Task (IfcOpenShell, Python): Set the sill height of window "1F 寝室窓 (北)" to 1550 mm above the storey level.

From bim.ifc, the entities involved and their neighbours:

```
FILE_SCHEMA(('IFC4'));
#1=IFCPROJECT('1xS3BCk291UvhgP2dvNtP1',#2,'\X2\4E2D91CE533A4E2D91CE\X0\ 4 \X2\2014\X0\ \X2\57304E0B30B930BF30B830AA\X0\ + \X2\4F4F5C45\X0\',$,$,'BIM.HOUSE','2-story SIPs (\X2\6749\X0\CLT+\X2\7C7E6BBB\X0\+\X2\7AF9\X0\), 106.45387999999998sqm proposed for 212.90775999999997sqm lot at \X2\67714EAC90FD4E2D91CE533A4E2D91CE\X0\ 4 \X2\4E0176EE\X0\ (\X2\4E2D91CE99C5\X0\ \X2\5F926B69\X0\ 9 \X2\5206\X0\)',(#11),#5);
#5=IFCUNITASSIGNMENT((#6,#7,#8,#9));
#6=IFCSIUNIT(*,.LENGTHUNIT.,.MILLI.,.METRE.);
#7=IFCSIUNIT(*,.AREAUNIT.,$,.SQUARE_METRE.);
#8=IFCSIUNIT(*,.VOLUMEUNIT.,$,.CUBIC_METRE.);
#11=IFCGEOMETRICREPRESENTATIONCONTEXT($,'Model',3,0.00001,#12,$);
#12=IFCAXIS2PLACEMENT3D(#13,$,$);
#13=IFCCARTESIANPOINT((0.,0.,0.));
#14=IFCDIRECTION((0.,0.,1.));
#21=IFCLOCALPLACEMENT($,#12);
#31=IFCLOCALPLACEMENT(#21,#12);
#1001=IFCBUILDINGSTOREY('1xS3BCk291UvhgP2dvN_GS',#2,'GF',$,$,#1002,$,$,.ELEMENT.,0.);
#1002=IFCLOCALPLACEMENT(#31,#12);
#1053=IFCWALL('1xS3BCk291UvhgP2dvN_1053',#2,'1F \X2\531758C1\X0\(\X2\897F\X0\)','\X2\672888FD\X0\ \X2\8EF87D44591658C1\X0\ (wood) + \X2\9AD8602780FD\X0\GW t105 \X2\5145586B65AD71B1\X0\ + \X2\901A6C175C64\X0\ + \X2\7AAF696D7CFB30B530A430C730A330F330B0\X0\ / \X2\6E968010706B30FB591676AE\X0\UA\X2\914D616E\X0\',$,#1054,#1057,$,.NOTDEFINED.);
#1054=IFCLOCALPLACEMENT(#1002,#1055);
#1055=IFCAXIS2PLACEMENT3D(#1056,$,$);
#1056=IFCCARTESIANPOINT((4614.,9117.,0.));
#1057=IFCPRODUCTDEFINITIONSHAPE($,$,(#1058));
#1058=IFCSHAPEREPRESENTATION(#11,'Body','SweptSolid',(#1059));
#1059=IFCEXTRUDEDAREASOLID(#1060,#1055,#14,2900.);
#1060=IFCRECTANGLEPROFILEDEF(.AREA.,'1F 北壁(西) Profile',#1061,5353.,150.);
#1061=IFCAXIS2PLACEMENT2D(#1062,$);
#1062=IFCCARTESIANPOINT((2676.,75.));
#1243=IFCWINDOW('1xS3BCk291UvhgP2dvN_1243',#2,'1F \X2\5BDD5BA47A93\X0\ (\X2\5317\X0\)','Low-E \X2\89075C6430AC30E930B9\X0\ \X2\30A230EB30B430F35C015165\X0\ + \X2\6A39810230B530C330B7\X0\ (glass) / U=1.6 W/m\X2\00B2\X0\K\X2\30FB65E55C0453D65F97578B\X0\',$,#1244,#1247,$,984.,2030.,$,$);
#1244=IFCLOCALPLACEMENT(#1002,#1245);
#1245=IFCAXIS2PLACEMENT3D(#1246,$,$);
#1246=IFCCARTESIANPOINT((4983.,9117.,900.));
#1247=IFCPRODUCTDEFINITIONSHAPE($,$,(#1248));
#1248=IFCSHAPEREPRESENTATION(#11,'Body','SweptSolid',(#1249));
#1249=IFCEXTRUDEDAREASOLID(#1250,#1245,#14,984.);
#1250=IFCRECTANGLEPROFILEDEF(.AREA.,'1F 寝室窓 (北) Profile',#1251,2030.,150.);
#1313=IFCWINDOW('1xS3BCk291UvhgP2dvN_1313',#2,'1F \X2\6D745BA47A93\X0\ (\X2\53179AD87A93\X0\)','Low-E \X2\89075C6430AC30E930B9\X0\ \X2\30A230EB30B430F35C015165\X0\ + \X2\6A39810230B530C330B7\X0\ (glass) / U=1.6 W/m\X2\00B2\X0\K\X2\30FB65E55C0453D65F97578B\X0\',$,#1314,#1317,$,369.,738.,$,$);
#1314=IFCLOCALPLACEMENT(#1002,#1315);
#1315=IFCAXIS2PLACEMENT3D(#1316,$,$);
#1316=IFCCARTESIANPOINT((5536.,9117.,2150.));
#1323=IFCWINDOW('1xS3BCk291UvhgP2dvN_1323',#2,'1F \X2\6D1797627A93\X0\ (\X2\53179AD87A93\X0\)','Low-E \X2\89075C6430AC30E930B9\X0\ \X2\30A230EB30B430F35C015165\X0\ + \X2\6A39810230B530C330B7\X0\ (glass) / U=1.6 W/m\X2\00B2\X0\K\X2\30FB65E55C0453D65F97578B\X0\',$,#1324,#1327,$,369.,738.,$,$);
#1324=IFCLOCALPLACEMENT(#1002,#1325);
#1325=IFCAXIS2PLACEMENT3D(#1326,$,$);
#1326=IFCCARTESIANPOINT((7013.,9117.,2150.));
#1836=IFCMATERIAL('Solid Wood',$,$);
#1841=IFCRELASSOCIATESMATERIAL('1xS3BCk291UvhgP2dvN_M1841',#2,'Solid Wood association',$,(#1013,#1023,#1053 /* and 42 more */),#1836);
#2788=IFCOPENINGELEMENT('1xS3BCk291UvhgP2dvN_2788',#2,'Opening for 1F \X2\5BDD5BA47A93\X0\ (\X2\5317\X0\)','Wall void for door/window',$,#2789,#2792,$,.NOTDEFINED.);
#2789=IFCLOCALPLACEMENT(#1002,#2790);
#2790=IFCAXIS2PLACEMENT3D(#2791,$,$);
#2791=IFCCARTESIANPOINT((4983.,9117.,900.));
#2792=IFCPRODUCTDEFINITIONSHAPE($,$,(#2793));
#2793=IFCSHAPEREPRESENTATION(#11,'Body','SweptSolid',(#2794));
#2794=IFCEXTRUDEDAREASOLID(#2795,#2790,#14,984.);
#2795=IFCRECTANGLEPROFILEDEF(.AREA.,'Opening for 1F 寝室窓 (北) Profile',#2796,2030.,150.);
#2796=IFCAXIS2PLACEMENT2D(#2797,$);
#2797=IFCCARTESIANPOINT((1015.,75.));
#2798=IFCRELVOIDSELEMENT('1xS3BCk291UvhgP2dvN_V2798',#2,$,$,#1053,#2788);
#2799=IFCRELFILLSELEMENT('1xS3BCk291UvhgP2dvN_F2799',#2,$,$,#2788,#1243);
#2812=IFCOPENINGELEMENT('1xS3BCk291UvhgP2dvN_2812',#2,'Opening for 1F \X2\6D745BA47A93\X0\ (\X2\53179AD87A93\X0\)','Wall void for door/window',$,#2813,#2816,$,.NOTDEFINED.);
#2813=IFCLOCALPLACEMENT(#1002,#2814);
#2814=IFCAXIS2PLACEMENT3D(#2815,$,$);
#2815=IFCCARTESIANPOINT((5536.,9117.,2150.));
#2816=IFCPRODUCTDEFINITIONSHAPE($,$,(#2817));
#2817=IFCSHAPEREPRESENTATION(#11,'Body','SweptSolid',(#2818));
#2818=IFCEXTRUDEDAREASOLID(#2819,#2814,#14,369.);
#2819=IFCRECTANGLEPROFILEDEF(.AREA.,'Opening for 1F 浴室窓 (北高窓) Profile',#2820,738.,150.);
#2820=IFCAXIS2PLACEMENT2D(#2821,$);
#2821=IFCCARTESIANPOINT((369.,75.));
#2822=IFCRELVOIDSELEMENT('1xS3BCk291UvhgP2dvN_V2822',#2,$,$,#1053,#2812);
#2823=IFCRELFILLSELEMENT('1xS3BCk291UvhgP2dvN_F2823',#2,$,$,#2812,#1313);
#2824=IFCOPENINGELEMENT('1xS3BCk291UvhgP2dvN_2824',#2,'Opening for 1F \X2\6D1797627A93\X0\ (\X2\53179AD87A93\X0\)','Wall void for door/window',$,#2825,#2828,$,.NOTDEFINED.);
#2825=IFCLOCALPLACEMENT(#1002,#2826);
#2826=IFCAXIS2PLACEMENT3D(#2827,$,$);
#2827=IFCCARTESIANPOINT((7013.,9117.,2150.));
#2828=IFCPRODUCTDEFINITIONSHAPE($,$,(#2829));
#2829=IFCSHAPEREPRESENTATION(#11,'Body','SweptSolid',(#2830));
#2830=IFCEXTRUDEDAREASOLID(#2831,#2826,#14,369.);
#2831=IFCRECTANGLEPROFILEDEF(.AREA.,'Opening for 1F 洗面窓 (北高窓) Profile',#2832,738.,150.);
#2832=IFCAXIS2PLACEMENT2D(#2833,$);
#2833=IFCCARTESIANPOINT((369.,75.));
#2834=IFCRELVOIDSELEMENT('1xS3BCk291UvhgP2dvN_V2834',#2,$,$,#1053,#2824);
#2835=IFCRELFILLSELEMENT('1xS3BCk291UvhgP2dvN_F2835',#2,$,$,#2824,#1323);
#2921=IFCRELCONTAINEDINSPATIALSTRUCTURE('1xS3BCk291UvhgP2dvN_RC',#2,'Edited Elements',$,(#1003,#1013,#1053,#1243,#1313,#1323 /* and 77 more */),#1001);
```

```python
import numpy as np
import ifcopenshell
import ifcopenshell.api.geometry
import ifcopenshell.geom
import ifcopenshell.util.element
import ifcopenshell.util.placement
import ifcopenshell.util.shape
import ifcopenshell.util.unit

model = ifcopenshell.open("bim.ifc")
unit_scale = ifcopenshell.util.unit.calculate_unit_scale(model)

window = model.by_guid("1xS3BCk291UvhgP2dvN_1243")
opening = window.FillsVoids[0].RelatingOpeningElement
storey = ifcopenshell.util.element.get_container(window, ifc_class="IfcBuildingStorey")
level = ifcopenshell.util.placement.get_local_placement(storey.ObjectPlacement)[2, 3]

# The opening's origin need not be at the sill, so measure its lowest point.
shape = ifcopenshell.geom.create_shape(ifcopenshell.geom.settings(), opening)
bottom = ifcopenshell.util.shape.get_shape_bottom_elevation(shape, shape.geometry) / unit_scale
dz = level + 1550.0 - bottom

shift = np.array([0.0, 0.0, dz])
# The window is not placed relative to its opening, so move both.
for product in (opening, window):
    matrix = ifcopenshell.util.placement.get_local_placement(product.ObjectPlacement)
    matrix[:3, 3] += shift
    ifcopenshell.api.geometry.edit_object_placement(model, product=product, matrix=matrix, is_si=False)

print(f"moved by {dz * unit_scale:+.3f} m")

model.write("bim_rev.ifc")
```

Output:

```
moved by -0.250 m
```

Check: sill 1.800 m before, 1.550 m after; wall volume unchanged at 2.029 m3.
